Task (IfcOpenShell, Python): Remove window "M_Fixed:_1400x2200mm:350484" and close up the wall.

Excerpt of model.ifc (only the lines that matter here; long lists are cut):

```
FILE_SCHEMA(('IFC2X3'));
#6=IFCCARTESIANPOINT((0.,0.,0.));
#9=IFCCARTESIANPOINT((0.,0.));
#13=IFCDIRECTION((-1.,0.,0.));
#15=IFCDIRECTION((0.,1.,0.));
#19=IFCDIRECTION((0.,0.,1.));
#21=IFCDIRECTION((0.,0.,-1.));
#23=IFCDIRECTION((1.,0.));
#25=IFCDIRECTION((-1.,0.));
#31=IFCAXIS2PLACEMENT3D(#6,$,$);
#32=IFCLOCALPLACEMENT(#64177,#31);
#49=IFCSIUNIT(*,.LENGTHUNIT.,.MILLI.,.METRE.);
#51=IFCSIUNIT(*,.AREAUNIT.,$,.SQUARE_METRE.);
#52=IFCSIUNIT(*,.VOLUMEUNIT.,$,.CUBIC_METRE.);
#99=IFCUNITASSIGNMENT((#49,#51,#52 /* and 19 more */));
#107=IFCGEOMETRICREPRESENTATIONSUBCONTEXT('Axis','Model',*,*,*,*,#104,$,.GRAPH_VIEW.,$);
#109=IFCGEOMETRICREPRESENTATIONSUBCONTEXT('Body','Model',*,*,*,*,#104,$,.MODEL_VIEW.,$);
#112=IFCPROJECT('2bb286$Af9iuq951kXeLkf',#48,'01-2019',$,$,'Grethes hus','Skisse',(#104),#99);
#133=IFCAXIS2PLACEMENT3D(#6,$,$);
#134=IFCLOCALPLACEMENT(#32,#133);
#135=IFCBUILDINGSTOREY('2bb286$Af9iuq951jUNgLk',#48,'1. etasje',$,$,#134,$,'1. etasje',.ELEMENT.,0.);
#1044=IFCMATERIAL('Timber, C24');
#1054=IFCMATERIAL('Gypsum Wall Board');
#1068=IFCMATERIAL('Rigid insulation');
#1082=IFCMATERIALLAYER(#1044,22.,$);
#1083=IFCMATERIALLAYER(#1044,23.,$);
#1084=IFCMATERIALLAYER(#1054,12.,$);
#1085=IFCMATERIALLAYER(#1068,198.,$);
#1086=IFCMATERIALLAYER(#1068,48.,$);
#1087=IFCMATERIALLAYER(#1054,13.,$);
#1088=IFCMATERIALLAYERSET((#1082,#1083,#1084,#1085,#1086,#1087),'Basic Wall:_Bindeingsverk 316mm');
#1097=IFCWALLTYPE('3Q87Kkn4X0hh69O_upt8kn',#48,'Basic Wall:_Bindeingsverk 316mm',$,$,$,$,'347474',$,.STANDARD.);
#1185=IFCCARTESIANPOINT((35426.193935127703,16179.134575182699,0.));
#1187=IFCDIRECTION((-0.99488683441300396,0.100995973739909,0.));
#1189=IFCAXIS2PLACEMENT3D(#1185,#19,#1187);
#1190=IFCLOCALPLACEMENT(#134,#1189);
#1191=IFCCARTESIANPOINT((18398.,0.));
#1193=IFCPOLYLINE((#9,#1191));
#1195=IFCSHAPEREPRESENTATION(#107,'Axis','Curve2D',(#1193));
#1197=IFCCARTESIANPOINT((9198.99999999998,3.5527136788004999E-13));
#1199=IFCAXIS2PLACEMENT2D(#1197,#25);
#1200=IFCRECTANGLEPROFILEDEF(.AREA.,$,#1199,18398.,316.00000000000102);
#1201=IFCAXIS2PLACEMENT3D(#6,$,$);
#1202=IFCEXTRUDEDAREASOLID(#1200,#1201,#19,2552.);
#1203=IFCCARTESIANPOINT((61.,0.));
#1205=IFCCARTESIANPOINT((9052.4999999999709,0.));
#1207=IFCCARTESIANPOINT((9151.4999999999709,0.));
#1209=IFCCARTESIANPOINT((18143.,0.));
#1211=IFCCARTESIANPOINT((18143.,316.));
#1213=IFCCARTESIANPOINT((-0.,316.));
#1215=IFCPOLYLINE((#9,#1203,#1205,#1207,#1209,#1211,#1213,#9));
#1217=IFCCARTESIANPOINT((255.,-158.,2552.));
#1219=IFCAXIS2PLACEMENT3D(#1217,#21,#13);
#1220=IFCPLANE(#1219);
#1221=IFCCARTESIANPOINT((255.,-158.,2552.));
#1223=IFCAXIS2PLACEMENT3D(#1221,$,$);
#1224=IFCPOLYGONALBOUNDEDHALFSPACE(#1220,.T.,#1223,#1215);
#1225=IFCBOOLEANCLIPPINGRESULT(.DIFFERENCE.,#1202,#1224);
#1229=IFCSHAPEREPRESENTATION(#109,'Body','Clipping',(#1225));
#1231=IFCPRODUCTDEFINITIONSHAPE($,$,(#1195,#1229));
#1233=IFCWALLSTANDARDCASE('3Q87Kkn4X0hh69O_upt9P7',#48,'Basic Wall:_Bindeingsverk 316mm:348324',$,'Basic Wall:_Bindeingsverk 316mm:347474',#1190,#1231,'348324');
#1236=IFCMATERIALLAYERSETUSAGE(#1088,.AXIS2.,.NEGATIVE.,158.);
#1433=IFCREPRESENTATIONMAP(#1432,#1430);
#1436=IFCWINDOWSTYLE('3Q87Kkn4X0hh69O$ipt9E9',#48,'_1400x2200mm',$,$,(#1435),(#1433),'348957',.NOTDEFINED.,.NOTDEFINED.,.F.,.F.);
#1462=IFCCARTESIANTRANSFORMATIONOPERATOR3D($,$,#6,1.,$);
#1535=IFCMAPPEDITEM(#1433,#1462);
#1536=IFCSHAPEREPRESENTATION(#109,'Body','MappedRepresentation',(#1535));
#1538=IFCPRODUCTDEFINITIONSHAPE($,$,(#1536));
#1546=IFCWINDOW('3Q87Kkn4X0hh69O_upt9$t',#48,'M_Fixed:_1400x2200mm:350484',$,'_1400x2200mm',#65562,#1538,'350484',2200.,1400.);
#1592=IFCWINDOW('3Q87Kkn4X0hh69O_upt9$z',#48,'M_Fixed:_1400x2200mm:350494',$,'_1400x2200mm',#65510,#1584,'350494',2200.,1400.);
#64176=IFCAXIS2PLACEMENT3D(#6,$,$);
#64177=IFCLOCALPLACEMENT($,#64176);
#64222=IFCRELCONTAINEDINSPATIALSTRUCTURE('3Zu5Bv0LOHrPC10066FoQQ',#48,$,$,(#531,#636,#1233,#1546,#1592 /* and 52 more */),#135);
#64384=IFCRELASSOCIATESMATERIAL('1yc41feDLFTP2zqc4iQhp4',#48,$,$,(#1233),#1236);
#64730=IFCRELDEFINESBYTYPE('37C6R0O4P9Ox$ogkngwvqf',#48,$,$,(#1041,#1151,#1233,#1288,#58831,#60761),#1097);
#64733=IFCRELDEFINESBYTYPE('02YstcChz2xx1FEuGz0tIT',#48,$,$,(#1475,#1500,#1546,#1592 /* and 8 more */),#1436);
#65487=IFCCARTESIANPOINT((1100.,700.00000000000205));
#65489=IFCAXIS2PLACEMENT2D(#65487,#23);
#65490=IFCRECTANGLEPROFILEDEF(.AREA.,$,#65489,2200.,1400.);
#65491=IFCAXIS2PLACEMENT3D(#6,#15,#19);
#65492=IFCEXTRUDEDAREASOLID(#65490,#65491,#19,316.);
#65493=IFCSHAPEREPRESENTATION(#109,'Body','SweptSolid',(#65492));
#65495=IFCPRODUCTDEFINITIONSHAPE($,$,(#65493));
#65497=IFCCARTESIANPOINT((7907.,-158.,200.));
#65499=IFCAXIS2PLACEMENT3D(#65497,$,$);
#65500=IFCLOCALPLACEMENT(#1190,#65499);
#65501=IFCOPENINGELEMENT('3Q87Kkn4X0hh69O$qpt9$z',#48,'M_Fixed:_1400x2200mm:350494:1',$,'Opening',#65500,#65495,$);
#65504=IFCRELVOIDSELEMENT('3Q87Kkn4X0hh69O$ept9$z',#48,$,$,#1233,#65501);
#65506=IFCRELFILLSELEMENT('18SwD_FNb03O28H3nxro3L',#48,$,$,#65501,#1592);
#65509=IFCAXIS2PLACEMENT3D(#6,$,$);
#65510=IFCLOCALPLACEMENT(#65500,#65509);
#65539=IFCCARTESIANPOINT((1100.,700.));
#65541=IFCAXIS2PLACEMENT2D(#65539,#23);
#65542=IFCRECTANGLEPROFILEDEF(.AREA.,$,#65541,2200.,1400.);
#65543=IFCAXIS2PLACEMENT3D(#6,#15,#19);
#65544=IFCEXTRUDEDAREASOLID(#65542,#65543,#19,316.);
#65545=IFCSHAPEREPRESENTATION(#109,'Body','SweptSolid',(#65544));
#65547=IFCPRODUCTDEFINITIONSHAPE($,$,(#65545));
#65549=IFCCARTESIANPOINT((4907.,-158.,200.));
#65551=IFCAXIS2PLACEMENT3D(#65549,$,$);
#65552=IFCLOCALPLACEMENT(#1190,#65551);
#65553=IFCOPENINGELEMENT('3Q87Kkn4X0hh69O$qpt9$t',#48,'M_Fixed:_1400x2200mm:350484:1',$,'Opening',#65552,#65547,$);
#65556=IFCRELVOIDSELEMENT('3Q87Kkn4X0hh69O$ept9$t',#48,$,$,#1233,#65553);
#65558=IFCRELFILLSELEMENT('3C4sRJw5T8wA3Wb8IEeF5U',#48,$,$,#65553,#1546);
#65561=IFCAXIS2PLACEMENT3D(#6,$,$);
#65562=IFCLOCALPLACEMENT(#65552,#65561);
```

```python
import ifcopenshell
import ifcopenshell.api.feature
import ifcopenshell.api.root
import ifcopenshell.geom
import ifcopenshell.util.shape

model = ifcopenshell.open("model.ifc")
settings = ifcopenshell.geom.settings()


def volume(element):
    """Net volume in cubic metres, openings subtracted."""
    shape = ifcopenshell.geom.create_shape(settings, element)
    return ifcopenshell.util.shape.get_volume(shape.geometry)


window = model.by_id(1546)
opening = window.FillsVoids[0].RelatingOpeningElement
wall = opening.VoidsElements[0].RelatingBuildingElement
before = volume(wall)

ifcopenshell.api.root.remove_product(model, product=window)
ifcopenshell.api.feature.remove_feature(model, feature=opening)

after = volume(wall)

print(f"wall volume {before:.3f} -> {after:.3f} m3")

model.write("model_updated.ifc")
```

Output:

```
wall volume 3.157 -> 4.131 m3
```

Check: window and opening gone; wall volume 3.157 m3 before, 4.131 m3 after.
